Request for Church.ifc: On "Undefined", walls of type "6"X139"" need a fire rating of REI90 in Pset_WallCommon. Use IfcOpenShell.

First a look at what the model holds.

```python
import ifcopenshell
import ifcopenshell.util.element

model = ifcopenshell.open("Church.ifc")
print(model.schema)
storey = next(s for s in model.by_type("IfcBuildingStorey") if s.Name == "Undefined")
walls = [e for e in ifcopenshell.util.element.get_decomposition(storey) if e.is_a("IfcWall")]
seen = {}
for e in walls:
    element_type = ifcopenshell.util.element.get_type(e)
    key = (element_type.Name if element_type != e and element_type else None, ifcopenshell.util.element.get_pset(e, "Pset_WallCommon", "FireRating"))
    seen[key] = seen.get(key, 0) + 1
for (name, value), count in sorted(seen.items(), key=str):
    print(count, "x", name, "|", value)
```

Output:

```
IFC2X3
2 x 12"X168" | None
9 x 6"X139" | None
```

```python
import ifcopenshell
import ifcopenshell.api.pset
import ifcopenshell.util.element

model = ifcopenshell.open("Church.ifc")

storey = next(s for s in model.by_type("IfcBuildingStorey") if s.Name == "Undefined")
walls = [e for e in ifcopenshell.util.element.get_decomposition(storey) if e.is_a("IfcWall")]

count = 0
for e in walls:
    element_type = ifcopenshell.util.element.get_type(e)
    if element_type in (None, e) or element_type.Name != '6"X139"':
        continue
    found = ifcopenshell.util.element.get_pset(e, "Pset_WallCommon", should_inherit=False)
    if found:
        pset = model.by_id(found["id"])
        if len(ifcopenshell.util.element.get_elements_by_pset(pset)) > 1:
            pset = ifcopenshell.api.pset.unshare_pset(model, products=[e], pset=pset)[0]
    else:
        pset = ifcopenshell.api.pset.add_pset(model, product=e, name="Pset_WallCommon")
    ifcopenshell.api.pset.edit_pset(model, pset=pset, properties={"FireRating": "REI90"})
    count += 1

print(count, "walls updated")

model.write("Church-out.ifc")
```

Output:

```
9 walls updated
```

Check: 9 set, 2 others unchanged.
